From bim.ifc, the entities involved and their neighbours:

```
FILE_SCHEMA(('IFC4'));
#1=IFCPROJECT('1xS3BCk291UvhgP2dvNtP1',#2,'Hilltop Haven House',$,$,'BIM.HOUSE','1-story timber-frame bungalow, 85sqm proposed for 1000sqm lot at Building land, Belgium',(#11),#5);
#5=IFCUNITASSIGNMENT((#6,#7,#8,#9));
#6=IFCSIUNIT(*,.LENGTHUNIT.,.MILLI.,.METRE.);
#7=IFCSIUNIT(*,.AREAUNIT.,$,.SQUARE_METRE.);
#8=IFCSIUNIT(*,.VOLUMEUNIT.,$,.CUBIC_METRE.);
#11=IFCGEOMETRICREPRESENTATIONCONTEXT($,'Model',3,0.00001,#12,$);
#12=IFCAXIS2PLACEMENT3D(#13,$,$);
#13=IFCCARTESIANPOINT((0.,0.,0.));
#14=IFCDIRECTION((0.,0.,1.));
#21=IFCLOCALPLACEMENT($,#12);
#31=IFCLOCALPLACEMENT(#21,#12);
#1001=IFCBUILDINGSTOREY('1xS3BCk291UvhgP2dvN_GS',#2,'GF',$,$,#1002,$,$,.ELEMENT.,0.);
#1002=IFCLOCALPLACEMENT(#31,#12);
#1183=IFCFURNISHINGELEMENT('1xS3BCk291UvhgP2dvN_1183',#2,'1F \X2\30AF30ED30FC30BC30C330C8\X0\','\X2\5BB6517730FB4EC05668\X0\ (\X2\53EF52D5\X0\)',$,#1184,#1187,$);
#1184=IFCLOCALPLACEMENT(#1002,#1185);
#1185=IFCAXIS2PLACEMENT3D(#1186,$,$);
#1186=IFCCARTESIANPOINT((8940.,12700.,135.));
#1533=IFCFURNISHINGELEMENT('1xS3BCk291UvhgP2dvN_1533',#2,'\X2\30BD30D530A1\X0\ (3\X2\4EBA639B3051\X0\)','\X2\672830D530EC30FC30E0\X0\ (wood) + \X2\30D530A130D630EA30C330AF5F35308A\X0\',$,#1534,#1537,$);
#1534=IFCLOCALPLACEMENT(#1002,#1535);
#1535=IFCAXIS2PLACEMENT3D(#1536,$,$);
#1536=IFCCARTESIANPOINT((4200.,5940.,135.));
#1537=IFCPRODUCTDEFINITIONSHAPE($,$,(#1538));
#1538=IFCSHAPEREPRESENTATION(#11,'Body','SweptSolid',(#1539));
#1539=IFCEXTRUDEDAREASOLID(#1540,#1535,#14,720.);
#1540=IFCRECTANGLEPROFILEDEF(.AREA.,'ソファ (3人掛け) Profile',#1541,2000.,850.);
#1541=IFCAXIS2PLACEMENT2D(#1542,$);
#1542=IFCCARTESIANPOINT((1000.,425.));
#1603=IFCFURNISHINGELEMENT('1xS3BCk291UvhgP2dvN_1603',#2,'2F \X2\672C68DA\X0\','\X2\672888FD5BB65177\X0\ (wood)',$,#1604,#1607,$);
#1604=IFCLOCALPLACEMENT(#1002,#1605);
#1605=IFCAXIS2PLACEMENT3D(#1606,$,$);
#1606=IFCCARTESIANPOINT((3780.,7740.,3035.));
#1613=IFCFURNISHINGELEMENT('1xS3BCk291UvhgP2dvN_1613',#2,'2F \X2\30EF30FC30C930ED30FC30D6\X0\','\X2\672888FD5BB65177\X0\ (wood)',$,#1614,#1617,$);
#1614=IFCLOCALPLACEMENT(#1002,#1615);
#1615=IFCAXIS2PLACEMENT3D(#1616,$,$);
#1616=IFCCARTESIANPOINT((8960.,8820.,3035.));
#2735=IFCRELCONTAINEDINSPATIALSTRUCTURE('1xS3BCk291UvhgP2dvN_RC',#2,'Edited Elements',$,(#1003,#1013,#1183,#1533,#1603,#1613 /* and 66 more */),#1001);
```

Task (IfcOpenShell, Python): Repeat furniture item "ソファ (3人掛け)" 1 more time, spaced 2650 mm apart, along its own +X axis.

```python
import ifcopenshell
import ifcopenshell.api.geometry
import ifcopenshell.api.root
import ifcopenshell.util.element
import ifcopenshell.util.placement
import ifcopenshell.util.unit

model = ifcopenshell.open("bim.ifc")
unit_scale = ifcopenshell.util.unit.calculate_unit_scale(model)


def reuse_history(source, copy):
    """copy_class also copies each property set's owner history, people and application; keep the originals."""
    for rel in copy.IsDefinedBy:
        if rel.is_a("IfcRelDefinesByProperties") and (history := rel.RelatingPropertyDefinition.OwnerHistory):
            rel.RelatingPropertyDefinition.OwnerHistory = source.OwnerHistory
            ifcopenshell.util.element.remove_deep2(model, history)


source = model.by_id(1533)
base = ifcopenshell.util.placement.get_local_placement(source.ObjectPlacement)
step = base[:3, 0] * 2.65 / unit_scale

for i in range(1, 2):
    copy = ifcopenshell.api.root.copy_class(model, product=source)
    copy.Representation = ifcopenshell.util.element.copy_deep(
        model, source.Representation, exclude=["IfcGeometricRepresentationContext", "IfcRepresentationMap"]
    )
    reuse_history(source, copy)
    matrix = base.copy()
    matrix[:3, 3] += i * step
    print("added at", matrix[:3, 3].round(3) + 0.0)
    ifcopenshell.api.geometry.edit_object_placement(model, product=copy, matrix=matrix, is_si=False)

model.write("bim_edited.ifc")
```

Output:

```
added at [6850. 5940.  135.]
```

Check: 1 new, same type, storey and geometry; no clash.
